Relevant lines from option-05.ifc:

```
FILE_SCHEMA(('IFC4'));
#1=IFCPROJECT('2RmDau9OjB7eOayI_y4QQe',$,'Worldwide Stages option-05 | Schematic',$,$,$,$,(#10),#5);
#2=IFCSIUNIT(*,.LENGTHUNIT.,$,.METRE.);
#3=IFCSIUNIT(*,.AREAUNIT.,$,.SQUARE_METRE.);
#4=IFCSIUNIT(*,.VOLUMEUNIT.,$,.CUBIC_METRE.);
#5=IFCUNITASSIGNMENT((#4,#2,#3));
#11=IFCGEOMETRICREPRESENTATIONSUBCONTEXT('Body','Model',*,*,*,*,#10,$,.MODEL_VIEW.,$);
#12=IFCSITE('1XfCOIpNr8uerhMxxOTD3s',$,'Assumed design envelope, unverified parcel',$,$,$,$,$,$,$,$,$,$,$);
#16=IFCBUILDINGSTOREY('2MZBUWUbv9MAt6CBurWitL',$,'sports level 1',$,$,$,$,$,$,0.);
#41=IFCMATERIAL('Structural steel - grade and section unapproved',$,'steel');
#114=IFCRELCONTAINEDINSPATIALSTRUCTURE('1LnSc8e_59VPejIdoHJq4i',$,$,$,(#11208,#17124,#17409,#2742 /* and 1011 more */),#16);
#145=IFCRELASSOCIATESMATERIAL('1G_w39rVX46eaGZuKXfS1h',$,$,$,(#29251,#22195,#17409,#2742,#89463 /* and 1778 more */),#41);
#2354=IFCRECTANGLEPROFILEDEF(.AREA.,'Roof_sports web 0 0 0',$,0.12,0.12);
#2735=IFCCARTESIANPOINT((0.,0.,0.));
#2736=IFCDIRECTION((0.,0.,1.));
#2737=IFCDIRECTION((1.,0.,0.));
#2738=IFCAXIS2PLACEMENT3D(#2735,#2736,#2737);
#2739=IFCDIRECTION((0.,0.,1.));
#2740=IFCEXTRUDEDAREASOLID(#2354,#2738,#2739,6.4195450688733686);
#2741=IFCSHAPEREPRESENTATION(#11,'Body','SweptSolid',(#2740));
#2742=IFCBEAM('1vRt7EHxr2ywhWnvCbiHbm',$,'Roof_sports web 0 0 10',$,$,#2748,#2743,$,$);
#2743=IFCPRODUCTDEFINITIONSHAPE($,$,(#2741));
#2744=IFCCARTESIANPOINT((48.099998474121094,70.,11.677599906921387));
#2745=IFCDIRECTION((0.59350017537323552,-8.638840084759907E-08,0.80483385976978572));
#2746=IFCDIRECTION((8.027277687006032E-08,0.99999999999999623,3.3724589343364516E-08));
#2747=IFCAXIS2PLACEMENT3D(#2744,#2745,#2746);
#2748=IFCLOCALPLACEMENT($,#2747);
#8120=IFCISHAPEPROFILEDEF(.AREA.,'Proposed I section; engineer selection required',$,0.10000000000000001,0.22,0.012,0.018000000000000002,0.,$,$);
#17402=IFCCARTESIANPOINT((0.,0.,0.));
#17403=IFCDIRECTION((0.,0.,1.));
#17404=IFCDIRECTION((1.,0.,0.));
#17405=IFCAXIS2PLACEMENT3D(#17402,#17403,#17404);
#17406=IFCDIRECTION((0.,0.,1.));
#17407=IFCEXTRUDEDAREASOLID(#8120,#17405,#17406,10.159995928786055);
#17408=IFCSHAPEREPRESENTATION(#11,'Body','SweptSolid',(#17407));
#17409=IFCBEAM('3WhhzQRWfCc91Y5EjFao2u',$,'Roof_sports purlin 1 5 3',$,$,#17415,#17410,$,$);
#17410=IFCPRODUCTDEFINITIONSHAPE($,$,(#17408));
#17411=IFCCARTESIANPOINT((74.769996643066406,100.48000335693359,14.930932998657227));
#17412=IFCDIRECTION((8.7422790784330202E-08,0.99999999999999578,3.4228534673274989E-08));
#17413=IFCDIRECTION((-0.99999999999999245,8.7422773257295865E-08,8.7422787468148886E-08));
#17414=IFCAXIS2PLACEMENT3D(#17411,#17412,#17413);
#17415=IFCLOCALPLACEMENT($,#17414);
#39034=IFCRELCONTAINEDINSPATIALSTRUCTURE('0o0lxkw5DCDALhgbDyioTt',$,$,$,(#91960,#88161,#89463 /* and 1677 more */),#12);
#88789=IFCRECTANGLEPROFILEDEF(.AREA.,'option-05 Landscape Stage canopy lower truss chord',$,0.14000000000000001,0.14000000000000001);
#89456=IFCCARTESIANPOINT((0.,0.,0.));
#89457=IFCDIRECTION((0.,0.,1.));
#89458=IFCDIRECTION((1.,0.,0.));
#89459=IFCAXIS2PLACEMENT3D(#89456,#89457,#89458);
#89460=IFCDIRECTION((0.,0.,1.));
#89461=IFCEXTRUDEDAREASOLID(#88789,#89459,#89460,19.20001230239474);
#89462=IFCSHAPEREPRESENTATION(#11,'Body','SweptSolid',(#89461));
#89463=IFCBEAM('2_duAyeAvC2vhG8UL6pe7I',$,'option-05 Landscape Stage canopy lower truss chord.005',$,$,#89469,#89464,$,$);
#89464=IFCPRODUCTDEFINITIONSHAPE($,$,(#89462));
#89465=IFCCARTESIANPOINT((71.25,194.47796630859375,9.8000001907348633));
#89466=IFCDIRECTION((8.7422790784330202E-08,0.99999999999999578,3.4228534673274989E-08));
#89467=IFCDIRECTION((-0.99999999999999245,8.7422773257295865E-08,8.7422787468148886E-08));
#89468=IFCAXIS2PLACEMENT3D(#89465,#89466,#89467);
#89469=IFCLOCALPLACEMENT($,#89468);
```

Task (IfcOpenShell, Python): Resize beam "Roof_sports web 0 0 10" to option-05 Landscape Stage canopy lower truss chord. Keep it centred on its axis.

```python
import ifcopenshell
import ifcopenshell.util.element
import ifcopenshell.util.representation

model = ifcopenshell.open("option-05.ifc")

member = model.by_guid("1vRt7EHxr2ywhWnvCbiHbm")
source = next(p for p in model.by_type("IfcRectangleProfileDef") if p.ProfileName == "option-05 Landscape Stage canopy lower truss chord")

body = ifcopenshell.util.representation.get_representation(member, "Model", "Body")
solid = body.Items[0]
old_profile = solid.SweptArea

# Copy the section's sizes but keep this member's own profile position.
profile = ifcopenshell.util.element.copy(model, source)
profile.Position = old_profile.Position
solid.SweptArea = profile
if not model.get_total_inverses(old_profile):
    ifcopenshell.util.element.remove_deep2(model, old_profile)

print(solid.SweptArea)

model.write("option-05_updated.ifc")
```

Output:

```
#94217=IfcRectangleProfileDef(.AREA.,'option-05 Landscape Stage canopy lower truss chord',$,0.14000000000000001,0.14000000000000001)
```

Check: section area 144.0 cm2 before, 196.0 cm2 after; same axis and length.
